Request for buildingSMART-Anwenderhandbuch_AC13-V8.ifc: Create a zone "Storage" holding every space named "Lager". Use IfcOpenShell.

First a look at what the model holds.

```python
import ifcopenshell

model = ifcopenshell.open("buildingSMART-Anwenderhandbuch_AC13-V8.ifc")
print(model.schema)
seen = {}
for space in model.by_type("IfcSpace"):
    seen[space.LongName] = seen.get(space.LongName, 0) + 1
for name, count in sorted(seen.items(), key=str):
    print(count, "x", name)
print("zones:", [z.Name for z in model.by_type("IfcZone")][:20])
```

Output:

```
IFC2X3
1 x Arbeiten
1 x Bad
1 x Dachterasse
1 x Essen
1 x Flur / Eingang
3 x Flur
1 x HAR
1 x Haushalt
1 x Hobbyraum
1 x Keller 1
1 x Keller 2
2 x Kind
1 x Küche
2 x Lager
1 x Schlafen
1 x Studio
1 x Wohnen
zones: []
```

```python
import ifcopenshell
import ifcopenshell.api.group
import ifcopenshell.api.root

model = ifcopenshell.open("buildingSMART-Anwenderhandbuch_AC13-V8.ifc")

names = {"Lager"}
spaces = [s for s in model.by_type("IfcSpace") if s.LongName in names]

zone = ifcopenshell.api.root.create_entity(model, ifc_class="IfcZone", name="Storage")
ifcopenshell.api.group.assign_group(model, products=spaces, group=zone)
print(len(spaces), "spaces in", zone.Name)

model.write("buildingSMART-Anwenderhandbuch_AC13-V8_rev.ifc")
```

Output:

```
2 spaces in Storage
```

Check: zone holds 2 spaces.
